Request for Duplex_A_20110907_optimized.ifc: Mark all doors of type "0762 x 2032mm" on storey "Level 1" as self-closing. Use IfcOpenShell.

First a look at what the model holds.

```python
import ifcopenshell
import ifcopenshell.util.element

model = ifcopenshell.open("Duplex_A_20110907_optimized.ifc")
print(model.schema)
storey = next(s for s in model.by_type("IfcBuildingStorey") if s.Name == "Level 1")
doors = [e for e in ifcopenshell.util.element.get_decomposition(storey) if e.is_a("IfcDoor")]
seen = {}
for e in doors:
    element_type = ifcopenshell.util.element.get_type(e)
    key = (element_type.Name if element_type != e and element_type else None, ifcopenshell.util.element.get_pset(e, "Pset_DoorCommon", "SelfClosing"))
    seen[key] = seen.get(key, 0) + 1
for (name, value), count in sorted(seen.items(), key=str):
    print(count, "x", name, "|", value)
```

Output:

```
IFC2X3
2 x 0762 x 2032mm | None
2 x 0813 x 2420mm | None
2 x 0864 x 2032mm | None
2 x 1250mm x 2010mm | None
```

```python
import ifcopenshell
import ifcopenshell.api.pset
import ifcopenshell.util.element

model = ifcopenshell.open("Duplex_A_20110907_optimized.ifc")

storey = next(s for s in model.by_type("IfcBuildingStorey") if s.Name == "Level 1")
doors = [e for e in ifcopenshell.util.element.get_decomposition(storey) if e.is_a("IfcDoor")]

count = 0
for e in doors:
    element_type = ifcopenshell.util.element.get_type(e)
    if element_type in (None, e) or element_type.Name != "0762 x 2032mm":
        continue
    # add_pset returns the element's existing set when there is one.
    pset = ifcopenshell.api.pset.add_pset(model, product=e, name="Pset_DoorCommon")
    ifcopenshell.api.pset.edit_pset(model, pset=pset, properties={"SelfClosing": True})
    count += 1

print(count, "doors updated")

model.write("Duplex_A_20110907_optimized-out.ifc")
```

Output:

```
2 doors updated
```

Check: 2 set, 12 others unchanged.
